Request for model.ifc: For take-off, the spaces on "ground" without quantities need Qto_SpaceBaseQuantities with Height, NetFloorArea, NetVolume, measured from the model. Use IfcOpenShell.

First a look at what the model holds.

```python
import ifcopenshell
import ifcopenshell.util.element
import ifcopenshell.util.unit

model = ifcopenshell.open("model.ifc")
print(model.schema)
for unit_type in ("LENGTHUNIT", "AREAUNIT", "VOLUMEUNIT"):
    print(unit_type, ifcopenshell.util.unit.calculate_unit_scale(model, unit_type))
storey = next(s for s in model.by_type("IfcBuildingStorey") if s.Name == "ground")
spaces = [e for e in ifcopenshell.util.element.get_decomposition(storey) if e.is_a("IfcSpace")]
for e in sorted(spaces, key=lambda e: e.id()):
    print(e.id(), e.is_a(), e.Name, list(ifcopenshell.util.element.get_psets(e, qtos_only=True)), sep=" | ")
```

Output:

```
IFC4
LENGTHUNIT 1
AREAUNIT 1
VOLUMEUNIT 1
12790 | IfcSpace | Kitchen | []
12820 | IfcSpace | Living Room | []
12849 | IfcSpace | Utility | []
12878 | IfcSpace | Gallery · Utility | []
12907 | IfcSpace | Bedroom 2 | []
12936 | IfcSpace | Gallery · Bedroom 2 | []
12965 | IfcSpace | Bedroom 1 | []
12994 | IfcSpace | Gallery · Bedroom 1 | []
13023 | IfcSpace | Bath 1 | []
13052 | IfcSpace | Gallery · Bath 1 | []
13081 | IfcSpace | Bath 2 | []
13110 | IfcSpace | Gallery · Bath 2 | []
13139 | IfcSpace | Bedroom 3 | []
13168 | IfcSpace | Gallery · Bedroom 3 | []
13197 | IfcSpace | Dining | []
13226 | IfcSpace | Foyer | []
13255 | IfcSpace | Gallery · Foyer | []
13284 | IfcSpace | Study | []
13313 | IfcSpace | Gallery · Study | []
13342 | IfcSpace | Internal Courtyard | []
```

```python
import ifcopenshell
import ifcopenshell.api.pset
import ifcopenshell.geom
import ifcopenshell.util.element
import ifcopenshell.util.shape
import ifcopenshell.util.unit

model = ifcopenshell.open("model.ifc")
unit_scale = ifcopenshell.util.unit.calculate_unit_scale(model)
area_scale = ifcopenshell.util.unit.calculate_unit_scale(model, "AREAUNIT")
volume_scale = ifcopenshell.util.unit.calculate_unit_scale(model, "VOLUMEUNIT")
settings = ifcopenshell.geom.settings()

storey = next(s for s in model.by_type("IfcBuildingStorey") if s.Name == "ground")
spaces = [e for e in ifcopenshell.util.element.get_decomposition(storey) if e.is_a("IfcSpace")]

for e in sorted(spaces, key=lambda e: e.id()):
    if ifcopenshell.util.element.get_psets(e, qtos_only=True, should_inherit=False):
        continue
    # Geometry comes back in metres, in the element's own axes.
    shape = ifcopenshell.geom.create_shape(settings, e)
    values = {
        "Height": ifcopenshell.util.shape.get_z(shape.geometry) / unit_scale,
        "NetFloorArea": ifcopenshell.util.shape.get_footprint_area(shape.geometry) / area_scale,
        "NetVolume": ifcopenshell.util.shape.get_volume(shape.geometry) / volume_scale,
    }
    qto = ifcopenshell.api.pset.add_qto(model, product=e, name="Qto_SpaceBaseQuantities")
    ifcopenshell.api.pset.edit_qto(model, qto=qto, properties=values)
    print(e.id(), {k: round(v, 3) for k, v in values.items()})

model.write("model_updated.ifc")
```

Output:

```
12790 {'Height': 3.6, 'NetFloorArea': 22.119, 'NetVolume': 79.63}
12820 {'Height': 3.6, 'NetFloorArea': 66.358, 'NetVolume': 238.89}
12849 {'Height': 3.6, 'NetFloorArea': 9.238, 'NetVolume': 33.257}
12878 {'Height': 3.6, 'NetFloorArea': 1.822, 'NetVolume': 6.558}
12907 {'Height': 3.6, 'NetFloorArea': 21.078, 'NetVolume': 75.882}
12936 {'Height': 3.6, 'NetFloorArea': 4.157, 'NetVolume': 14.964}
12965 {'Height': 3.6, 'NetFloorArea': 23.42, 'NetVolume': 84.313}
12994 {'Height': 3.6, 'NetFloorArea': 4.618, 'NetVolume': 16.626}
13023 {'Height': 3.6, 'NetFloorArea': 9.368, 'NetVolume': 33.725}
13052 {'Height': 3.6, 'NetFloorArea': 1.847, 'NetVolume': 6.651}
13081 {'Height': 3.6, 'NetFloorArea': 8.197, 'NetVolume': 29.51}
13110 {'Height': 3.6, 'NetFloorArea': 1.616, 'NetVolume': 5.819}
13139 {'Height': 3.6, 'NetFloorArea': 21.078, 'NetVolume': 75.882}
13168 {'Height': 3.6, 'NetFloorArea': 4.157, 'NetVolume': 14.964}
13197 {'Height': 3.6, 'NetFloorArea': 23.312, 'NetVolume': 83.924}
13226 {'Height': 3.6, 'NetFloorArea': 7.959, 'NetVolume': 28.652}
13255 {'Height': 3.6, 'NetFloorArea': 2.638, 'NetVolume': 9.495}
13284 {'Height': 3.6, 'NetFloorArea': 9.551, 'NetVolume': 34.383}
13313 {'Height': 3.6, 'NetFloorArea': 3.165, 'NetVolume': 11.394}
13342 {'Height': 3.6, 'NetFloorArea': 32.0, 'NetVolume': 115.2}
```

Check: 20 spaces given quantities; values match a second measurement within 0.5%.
